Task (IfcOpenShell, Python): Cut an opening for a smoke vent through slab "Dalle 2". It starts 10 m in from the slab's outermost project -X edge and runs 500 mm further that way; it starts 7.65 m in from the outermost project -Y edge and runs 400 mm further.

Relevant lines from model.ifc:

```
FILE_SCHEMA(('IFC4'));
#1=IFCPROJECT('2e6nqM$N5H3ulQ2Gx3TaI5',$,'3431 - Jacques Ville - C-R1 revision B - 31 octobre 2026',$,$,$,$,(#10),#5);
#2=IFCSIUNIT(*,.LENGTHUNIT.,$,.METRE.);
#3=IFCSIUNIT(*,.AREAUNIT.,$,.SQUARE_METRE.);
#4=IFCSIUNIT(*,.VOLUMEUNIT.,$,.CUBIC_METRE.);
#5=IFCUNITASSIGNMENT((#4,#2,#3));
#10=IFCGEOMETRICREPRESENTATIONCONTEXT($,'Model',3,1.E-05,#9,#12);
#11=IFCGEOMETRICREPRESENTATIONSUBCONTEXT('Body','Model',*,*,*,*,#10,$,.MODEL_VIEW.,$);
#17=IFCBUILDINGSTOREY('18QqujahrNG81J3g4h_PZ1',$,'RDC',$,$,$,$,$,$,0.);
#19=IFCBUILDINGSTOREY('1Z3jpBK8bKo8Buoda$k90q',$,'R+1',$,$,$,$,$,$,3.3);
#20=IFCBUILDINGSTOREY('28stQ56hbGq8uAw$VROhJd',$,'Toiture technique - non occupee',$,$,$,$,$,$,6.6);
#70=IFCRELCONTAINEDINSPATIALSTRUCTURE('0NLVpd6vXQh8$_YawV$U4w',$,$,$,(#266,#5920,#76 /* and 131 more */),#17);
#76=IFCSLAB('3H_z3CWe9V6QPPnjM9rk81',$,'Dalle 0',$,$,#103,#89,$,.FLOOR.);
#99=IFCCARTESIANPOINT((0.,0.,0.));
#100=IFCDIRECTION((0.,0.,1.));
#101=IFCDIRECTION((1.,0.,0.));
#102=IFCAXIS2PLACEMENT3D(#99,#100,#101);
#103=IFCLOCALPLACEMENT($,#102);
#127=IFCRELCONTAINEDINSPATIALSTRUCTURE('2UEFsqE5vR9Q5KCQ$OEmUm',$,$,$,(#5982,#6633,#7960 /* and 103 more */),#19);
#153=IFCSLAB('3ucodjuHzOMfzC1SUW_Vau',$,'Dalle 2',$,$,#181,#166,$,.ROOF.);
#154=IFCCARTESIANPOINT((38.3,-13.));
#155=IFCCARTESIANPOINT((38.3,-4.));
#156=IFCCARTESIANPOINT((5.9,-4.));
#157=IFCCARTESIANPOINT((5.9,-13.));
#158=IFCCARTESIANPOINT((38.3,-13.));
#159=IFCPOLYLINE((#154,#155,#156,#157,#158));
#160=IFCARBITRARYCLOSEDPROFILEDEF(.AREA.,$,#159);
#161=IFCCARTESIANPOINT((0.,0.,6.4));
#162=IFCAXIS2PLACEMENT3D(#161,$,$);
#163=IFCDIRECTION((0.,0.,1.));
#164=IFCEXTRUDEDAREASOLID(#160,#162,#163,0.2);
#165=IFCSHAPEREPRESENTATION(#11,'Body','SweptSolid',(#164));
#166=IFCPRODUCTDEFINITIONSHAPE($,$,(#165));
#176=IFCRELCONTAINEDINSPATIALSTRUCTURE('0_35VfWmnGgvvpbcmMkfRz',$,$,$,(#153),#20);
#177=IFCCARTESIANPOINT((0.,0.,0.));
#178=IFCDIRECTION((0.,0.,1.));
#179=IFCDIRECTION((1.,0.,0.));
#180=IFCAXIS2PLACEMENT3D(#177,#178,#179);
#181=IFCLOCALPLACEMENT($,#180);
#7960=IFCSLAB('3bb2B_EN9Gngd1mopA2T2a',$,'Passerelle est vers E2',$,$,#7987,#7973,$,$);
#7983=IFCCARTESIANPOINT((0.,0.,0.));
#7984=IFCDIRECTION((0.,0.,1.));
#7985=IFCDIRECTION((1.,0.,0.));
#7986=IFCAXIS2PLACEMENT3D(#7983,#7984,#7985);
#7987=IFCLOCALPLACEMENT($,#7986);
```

```python
import numpy as np
import ifcopenshell
import ifcopenshell.api.feature
import ifcopenshell.api.geometry
import ifcopenshell.api.root
import ifcopenshell.geom
import ifcopenshell.util.placement
import ifcopenshell.util.representation
import ifcopenshell.util.shape
import ifcopenshell.util.unit

model = ifcopenshell.open("model.ifc")
unit_scale = ifcopenshell.util.unit.calculate_unit_scale(model)
settings = ifcopenshell.geom.settings()


def volume(element):
    """Net volume in cubic metres, openings subtracted."""
    shape = ifcopenshell.geom.create_shape(settings, element)
    return ifcopenshell.util.shape.get_volume(shape.geometry)


slab = model.by_id(153)
before = volume(slab)

# Extent in the slab's own axes, in metres. The edges named are its -X and -Y sides.
slab_shape = ifcopenshell.geom.create_shape(settings, slab)
vertices = ifcopenshell.util.shape.get_vertices(slab_shape.geometry)
x_min, y_min, bottom = vertices.min(axis=0)
top = vertices[:, 2].max()

opening = ifcopenshell.api.root.create_entity(model, ifc_class="IfcOpeningElement", name="Smoke vent opening", predefined_type="OPENING")
context = ifcopenshell.util.representation.get_context(model, "Model", "Body", "MODEL_VIEW")
width, depth = 0.5, 0.4
outline = [(0.0, 0.0), (width, 0.0), (width, depth), (0.0, depth), (0.0, 0.0)]
# Overshoot both faces by 50 mm so the cut is clean.
shape = ifcopenshell.api.geometry.add_slab_representation(
    model, context=context, depth=top - bottom + 0.1, polyline=outline
)
ifcopenshell.api.geometry.assign_representation(model, product=opening, representation=shape)

matrix = ifcopenshell.util.placement.get_local_placement(slab.ObjectPlacement)
matrix[:, 3] = matrix @ np.append(np.array([x_min + 10, y_min + 7.65, bottom - 0.05]) / unit_scale, 1.0)
ifcopenshell.api.geometry.edit_object_placement(model, product=opening, matrix=matrix, is_si=False)
ifcopenshell.api.feature.add_feature(model, feature=opening, element=slab)

after = volume(slab)

print(f"slab volume {before:.3f} -> {after:.3f} m3")

model.write("model_v2.ifc")
```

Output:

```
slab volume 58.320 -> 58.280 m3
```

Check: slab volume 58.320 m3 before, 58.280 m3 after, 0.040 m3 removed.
